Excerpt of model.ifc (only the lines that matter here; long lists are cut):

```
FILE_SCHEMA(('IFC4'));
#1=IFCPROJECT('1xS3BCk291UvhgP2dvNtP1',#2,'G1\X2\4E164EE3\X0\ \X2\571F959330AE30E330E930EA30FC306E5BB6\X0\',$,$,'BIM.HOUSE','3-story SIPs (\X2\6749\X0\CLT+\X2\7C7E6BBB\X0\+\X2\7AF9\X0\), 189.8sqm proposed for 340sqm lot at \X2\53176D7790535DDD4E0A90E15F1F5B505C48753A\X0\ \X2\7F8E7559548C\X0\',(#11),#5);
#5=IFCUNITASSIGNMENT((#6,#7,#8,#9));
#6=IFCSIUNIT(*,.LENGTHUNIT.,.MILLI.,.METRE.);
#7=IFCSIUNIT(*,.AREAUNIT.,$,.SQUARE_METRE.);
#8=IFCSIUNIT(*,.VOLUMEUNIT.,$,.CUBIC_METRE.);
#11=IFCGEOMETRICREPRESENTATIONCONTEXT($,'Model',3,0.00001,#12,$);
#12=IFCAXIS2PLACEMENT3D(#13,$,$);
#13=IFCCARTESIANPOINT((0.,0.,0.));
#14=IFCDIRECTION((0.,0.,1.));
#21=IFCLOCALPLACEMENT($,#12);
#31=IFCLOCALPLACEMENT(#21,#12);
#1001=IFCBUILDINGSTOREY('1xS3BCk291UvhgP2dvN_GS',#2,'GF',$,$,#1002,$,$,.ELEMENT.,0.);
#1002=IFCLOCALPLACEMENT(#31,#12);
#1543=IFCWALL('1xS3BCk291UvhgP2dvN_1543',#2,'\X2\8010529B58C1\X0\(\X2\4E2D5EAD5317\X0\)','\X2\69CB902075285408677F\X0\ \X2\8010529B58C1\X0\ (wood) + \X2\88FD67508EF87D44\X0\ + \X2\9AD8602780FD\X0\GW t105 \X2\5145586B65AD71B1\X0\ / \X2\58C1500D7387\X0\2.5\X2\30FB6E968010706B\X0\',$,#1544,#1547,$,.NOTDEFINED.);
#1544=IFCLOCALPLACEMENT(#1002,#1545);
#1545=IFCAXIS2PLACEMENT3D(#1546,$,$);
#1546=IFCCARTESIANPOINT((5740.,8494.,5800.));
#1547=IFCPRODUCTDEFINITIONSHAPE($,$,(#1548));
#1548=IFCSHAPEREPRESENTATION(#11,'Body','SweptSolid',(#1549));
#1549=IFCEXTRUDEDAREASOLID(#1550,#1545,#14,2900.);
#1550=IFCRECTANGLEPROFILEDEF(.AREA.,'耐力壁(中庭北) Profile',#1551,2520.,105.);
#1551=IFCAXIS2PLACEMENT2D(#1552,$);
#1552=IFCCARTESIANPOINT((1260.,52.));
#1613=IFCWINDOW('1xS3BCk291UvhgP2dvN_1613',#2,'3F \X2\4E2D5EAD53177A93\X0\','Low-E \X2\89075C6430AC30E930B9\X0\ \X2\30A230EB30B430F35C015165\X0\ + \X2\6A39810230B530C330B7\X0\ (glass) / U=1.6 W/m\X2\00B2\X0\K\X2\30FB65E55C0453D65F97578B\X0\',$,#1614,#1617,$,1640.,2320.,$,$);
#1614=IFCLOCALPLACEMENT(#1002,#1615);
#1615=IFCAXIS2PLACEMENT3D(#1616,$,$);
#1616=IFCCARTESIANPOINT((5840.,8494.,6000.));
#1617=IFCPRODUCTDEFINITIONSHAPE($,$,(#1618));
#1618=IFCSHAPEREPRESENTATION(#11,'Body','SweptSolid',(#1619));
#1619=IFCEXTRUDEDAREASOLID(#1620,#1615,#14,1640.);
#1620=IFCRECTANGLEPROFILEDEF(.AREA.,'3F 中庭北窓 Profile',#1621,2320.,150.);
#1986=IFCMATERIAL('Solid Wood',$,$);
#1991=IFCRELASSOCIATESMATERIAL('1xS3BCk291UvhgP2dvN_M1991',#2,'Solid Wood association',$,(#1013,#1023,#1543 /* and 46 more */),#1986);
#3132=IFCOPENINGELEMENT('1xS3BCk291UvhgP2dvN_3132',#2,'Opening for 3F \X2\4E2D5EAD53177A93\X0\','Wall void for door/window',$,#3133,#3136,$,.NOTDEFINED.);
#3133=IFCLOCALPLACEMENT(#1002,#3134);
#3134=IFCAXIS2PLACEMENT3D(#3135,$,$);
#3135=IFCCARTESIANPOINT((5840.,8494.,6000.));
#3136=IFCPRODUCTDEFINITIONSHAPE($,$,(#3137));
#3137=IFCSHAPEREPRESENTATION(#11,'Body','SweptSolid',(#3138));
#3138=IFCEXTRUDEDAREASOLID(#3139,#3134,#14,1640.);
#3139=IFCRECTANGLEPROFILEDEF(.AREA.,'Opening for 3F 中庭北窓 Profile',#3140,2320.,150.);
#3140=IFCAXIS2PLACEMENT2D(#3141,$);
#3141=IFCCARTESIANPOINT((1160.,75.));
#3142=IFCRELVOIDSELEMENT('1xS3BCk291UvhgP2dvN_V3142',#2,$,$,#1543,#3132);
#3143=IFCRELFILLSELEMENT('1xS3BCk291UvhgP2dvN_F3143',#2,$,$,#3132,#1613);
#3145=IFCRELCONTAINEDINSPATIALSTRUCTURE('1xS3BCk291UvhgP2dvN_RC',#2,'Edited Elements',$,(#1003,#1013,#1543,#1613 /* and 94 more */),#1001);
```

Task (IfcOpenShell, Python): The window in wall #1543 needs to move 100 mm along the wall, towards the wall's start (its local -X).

```python
import ifcopenshell
import ifcopenshell.api.geometry
import ifcopenshell.util.placement
import ifcopenshell.util.unit

model = ifcopenshell.open("model.ifc")
unit_scale = ifcopenshell.util.unit.calculate_unit_scale(model)

window = model.by_guid("1xS3BCk291UvhgP2dvN_1613")
opening = window.FillsVoids[0].RelatingOpeningElement
wall = opening.VoidsElements[0].RelatingBuildingElement

wall_matrix = ifcopenshell.util.placement.get_local_placement(wall.ObjectPlacement)
shift = wall_matrix[:3, 0] * -0.1 / unit_scale
before = ifcopenshell.util.placement.get_local_placement(window.ObjectPlacement)[:3, 3].copy()

# The window is not placed relative to its opening, so move both.
for product in (opening, window):
    matrix = ifcopenshell.util.placement.get_local_placement(product.ObjectPlacement)
    matrix[:3, 3] += shift
    ifcopenshell.api.geometry.edit_object_placement(model, product=product, matrix=matrix, is_si=False)

after = ifcopenshell.util.placement.get_local_placement(window.ObjectPlacement)[:3, 3]
print("window moved by", (after - before).round(3) + 0.0)

model.write("model_v2.ifc")
```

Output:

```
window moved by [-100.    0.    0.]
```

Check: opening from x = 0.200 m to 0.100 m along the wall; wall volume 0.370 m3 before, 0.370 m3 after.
